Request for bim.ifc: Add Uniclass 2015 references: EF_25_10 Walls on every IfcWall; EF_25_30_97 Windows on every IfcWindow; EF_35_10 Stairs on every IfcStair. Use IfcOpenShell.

First a look at what the model holds.

```python
import ifcopenshell

model = ifcopenshell.open("bim.ifc")
print(model.schema)
print("classifications:", [c.Name for c in model.by_type("IfcClassification")])
for ifc_class in ("IfcDoor", "IfcRoof", "IfcStair", "IfcWall", "IfcWindow"):
    print(ifc_class, len(model.by_type(ifc_class)))
```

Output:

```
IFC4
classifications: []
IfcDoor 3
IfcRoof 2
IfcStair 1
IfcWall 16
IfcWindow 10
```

```python
import ifcopenshell
import ifcopenshell.api.classification

model = ifcopenshell.open("bim.ifc")

system = ifcopenshell.api.classification.add_classification(model, classification="Uniclass 2015")

codes = {
    "IfcWall": ("EF_25_10", "Walls"),
    "IfcWindow": ("EF_25_30_97", "Windows"),
    "IfcStair": ("EF_35_10", "Stairs"),
}
for ifc_class, (code, name) in codes.items():
    products = model.by_type(ifc_class)
    ifcopenshell.api.classification.add_reference(
        model, products=products, classification=system, identification=code, name=name
    )
    print(code, len(products))

model.write("bim_rev.ifc")
```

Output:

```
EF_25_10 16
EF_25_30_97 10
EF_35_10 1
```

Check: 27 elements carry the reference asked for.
